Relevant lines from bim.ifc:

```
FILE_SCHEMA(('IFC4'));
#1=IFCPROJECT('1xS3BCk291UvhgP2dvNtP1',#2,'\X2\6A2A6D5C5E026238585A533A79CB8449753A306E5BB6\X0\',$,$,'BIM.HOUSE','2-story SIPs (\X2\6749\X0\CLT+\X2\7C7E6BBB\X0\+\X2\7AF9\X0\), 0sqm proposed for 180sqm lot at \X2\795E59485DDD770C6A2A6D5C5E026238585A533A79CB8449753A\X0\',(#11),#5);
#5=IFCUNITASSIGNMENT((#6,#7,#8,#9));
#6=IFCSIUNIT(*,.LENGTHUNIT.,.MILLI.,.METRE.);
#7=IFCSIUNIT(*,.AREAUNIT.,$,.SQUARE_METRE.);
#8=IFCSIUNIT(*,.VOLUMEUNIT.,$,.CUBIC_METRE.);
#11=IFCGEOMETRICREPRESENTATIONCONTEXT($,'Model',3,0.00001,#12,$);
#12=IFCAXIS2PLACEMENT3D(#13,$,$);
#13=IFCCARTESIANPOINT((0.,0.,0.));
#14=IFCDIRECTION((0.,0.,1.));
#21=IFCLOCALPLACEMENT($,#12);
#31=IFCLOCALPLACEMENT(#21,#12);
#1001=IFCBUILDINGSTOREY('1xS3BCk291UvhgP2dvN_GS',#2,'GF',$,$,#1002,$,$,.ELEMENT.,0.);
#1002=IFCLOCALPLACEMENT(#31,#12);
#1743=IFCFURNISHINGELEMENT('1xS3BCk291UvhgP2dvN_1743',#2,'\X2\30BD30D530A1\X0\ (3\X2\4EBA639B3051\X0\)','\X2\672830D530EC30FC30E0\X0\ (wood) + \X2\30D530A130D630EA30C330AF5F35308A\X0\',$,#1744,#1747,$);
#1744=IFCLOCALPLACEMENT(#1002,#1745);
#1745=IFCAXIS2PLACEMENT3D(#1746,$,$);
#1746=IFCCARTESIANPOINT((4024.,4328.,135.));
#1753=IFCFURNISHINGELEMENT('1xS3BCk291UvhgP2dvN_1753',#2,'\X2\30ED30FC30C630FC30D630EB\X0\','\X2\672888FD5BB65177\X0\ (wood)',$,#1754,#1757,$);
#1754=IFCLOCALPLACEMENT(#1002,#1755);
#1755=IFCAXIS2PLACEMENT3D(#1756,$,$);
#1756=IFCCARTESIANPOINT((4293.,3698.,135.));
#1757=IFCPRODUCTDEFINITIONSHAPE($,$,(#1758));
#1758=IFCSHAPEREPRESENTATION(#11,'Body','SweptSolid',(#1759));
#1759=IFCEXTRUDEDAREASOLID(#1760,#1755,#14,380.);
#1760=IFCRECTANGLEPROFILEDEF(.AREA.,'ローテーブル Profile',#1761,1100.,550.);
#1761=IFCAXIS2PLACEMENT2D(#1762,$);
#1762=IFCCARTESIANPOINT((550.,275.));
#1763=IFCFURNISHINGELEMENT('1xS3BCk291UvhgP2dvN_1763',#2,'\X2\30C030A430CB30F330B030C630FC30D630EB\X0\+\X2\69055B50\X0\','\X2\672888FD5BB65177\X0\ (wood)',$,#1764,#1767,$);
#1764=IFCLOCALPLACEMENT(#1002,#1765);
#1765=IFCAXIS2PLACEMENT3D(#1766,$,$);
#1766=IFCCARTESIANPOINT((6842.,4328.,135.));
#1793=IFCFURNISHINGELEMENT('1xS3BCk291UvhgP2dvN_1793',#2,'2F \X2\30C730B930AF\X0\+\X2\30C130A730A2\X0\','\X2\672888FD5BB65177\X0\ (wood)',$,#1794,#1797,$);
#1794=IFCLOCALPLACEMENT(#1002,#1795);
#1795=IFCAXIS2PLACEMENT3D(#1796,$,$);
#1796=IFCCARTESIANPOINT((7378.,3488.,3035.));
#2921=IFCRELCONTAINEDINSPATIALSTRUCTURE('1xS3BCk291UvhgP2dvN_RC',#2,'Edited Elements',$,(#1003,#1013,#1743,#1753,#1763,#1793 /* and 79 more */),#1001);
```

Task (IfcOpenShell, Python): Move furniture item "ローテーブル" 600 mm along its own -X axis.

```python
import ifcopenshell
import ifcopenshell.api.geometry
import ifcopenshell.util.placement
import ifcopenshell.util.unit

model = ifcopenshell.open("bim.ifc")
unit_scale = ifcopenshell.util.unit.calculate_unit_scale(model)

item = model.by_id(1753)
matrix = ifcopenshell.util.placement.get_local_placement(item.ObjectPlacement)
matrix[:3, 3] -= matrix[:3, 0] * 0.6 / unit_scale
ifcopenshell.api.geometry.edit_object_placement(model, product=item, matrix=matrix, is_si=False)

print(ifcopenshell.util.placement.get_local_placement(item.ObjectPlacement).round(3) + 0.0)

model.write("bim_edited.ifc")
```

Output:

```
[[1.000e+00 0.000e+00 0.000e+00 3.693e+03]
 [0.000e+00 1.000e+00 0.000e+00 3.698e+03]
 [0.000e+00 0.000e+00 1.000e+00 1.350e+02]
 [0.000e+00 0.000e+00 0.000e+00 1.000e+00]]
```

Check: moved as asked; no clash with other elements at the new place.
